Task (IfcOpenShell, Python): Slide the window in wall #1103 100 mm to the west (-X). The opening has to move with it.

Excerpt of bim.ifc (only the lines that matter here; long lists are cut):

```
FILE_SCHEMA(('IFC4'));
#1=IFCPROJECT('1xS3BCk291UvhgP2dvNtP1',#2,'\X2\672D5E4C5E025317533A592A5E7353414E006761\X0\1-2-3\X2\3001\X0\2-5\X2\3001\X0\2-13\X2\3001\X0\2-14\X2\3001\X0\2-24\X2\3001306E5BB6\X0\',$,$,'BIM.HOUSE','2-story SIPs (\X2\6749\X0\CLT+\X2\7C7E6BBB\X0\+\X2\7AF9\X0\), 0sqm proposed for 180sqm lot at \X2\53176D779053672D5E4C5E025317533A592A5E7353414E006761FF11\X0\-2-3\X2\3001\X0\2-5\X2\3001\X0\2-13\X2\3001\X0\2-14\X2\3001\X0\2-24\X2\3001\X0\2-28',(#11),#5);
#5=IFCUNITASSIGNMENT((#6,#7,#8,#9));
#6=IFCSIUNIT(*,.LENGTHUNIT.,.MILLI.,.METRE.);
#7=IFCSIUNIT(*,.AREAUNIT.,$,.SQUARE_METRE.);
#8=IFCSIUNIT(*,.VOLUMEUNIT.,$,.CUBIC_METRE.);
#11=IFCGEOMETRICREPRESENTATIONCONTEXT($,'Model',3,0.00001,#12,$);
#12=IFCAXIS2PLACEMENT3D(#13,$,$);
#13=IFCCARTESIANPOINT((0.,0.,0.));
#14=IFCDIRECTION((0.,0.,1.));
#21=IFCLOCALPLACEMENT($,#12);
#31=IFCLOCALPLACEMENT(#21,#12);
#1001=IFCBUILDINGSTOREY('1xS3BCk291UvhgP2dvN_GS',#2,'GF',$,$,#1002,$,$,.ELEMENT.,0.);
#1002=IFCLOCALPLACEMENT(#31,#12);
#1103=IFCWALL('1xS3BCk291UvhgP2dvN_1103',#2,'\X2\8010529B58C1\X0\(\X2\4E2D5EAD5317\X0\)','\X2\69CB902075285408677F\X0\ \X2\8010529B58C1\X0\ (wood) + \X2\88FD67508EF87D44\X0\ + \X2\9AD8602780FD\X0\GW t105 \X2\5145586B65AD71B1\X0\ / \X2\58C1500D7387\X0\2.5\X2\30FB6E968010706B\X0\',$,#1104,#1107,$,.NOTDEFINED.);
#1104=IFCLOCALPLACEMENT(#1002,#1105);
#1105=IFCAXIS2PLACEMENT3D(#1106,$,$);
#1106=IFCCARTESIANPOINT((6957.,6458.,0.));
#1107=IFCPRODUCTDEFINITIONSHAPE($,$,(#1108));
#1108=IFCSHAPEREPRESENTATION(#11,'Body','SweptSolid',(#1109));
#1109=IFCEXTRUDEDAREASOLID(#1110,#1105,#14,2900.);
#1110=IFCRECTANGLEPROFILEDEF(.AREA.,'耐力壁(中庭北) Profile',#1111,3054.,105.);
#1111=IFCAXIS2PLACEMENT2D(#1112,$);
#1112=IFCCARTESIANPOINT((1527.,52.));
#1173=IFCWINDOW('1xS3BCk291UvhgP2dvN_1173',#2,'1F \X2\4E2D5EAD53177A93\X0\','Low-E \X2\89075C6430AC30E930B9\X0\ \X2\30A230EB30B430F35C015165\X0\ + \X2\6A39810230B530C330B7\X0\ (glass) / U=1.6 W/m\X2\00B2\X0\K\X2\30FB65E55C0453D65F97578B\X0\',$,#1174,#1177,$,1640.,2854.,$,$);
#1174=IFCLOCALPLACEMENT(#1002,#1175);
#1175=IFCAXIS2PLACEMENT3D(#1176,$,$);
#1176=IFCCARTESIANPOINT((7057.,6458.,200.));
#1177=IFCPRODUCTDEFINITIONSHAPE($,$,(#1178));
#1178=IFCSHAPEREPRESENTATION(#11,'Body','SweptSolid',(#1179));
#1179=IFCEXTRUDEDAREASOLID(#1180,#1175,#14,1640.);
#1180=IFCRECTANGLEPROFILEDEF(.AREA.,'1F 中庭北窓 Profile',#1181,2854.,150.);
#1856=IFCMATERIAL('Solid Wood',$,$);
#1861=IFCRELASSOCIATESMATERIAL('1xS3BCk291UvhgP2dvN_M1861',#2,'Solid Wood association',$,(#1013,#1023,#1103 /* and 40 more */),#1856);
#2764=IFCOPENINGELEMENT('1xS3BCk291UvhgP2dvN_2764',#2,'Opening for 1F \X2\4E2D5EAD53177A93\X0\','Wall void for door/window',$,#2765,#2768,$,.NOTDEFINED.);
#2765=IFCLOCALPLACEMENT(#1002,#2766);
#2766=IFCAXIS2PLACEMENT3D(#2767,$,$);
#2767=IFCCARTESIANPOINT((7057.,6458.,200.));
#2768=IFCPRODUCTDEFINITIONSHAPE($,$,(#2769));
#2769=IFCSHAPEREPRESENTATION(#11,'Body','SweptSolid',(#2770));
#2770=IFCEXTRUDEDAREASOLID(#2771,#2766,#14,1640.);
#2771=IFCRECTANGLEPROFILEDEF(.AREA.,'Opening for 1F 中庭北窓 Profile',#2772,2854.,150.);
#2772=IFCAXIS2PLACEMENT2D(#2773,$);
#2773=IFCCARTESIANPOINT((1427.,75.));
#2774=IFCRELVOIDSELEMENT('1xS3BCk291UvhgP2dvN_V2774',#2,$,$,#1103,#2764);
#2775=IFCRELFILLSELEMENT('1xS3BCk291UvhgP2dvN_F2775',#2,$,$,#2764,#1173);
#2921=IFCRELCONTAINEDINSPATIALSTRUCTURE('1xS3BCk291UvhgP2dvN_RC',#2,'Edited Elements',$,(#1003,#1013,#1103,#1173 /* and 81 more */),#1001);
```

```python
import ifcopenshell
import ifcopenshell.api.geometry
import ifcopenshell.util.placement

model = ifcopenshell.open("bim.ifc")

window = model.by_guid("1xS3BCk291UvhgP2dvN_1173")
opening = window.FillsVoids[0].RelatingOpeningElement
wall = opening.VoidsElements[0].RelatingBuildingElement

wall_matrix = ifcopenshell.util.placement.get_local_placement(wall.ObjectPlacement)
shift = wall_matrix[:3, 0] * -100.0
before = ifcopenshell.util.placement.get_local_placement(window.ObjectPlacement)[:3, 3].copy()

# The window is not placed relative to its opening, so move both.
for product in (opening, window):
    matrix = ifcopenshell.util.placement.get_local_placement(product.ObjectPlacement)
    matrix[:3, 3] += shift
    ifcopenshell.api.geometry.edit_object_placement(model, product=product, matrix=matrix, is_si=False)

after = ifcopenshell.util.placement.get_local_placement(window.ObjectPlacement)[:3, 3]
print("window moved by", (after - before).round(3) + 0.0)

model.write("bim_v2.ifc")
```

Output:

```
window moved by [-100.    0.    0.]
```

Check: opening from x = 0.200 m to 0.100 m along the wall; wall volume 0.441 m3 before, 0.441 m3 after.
